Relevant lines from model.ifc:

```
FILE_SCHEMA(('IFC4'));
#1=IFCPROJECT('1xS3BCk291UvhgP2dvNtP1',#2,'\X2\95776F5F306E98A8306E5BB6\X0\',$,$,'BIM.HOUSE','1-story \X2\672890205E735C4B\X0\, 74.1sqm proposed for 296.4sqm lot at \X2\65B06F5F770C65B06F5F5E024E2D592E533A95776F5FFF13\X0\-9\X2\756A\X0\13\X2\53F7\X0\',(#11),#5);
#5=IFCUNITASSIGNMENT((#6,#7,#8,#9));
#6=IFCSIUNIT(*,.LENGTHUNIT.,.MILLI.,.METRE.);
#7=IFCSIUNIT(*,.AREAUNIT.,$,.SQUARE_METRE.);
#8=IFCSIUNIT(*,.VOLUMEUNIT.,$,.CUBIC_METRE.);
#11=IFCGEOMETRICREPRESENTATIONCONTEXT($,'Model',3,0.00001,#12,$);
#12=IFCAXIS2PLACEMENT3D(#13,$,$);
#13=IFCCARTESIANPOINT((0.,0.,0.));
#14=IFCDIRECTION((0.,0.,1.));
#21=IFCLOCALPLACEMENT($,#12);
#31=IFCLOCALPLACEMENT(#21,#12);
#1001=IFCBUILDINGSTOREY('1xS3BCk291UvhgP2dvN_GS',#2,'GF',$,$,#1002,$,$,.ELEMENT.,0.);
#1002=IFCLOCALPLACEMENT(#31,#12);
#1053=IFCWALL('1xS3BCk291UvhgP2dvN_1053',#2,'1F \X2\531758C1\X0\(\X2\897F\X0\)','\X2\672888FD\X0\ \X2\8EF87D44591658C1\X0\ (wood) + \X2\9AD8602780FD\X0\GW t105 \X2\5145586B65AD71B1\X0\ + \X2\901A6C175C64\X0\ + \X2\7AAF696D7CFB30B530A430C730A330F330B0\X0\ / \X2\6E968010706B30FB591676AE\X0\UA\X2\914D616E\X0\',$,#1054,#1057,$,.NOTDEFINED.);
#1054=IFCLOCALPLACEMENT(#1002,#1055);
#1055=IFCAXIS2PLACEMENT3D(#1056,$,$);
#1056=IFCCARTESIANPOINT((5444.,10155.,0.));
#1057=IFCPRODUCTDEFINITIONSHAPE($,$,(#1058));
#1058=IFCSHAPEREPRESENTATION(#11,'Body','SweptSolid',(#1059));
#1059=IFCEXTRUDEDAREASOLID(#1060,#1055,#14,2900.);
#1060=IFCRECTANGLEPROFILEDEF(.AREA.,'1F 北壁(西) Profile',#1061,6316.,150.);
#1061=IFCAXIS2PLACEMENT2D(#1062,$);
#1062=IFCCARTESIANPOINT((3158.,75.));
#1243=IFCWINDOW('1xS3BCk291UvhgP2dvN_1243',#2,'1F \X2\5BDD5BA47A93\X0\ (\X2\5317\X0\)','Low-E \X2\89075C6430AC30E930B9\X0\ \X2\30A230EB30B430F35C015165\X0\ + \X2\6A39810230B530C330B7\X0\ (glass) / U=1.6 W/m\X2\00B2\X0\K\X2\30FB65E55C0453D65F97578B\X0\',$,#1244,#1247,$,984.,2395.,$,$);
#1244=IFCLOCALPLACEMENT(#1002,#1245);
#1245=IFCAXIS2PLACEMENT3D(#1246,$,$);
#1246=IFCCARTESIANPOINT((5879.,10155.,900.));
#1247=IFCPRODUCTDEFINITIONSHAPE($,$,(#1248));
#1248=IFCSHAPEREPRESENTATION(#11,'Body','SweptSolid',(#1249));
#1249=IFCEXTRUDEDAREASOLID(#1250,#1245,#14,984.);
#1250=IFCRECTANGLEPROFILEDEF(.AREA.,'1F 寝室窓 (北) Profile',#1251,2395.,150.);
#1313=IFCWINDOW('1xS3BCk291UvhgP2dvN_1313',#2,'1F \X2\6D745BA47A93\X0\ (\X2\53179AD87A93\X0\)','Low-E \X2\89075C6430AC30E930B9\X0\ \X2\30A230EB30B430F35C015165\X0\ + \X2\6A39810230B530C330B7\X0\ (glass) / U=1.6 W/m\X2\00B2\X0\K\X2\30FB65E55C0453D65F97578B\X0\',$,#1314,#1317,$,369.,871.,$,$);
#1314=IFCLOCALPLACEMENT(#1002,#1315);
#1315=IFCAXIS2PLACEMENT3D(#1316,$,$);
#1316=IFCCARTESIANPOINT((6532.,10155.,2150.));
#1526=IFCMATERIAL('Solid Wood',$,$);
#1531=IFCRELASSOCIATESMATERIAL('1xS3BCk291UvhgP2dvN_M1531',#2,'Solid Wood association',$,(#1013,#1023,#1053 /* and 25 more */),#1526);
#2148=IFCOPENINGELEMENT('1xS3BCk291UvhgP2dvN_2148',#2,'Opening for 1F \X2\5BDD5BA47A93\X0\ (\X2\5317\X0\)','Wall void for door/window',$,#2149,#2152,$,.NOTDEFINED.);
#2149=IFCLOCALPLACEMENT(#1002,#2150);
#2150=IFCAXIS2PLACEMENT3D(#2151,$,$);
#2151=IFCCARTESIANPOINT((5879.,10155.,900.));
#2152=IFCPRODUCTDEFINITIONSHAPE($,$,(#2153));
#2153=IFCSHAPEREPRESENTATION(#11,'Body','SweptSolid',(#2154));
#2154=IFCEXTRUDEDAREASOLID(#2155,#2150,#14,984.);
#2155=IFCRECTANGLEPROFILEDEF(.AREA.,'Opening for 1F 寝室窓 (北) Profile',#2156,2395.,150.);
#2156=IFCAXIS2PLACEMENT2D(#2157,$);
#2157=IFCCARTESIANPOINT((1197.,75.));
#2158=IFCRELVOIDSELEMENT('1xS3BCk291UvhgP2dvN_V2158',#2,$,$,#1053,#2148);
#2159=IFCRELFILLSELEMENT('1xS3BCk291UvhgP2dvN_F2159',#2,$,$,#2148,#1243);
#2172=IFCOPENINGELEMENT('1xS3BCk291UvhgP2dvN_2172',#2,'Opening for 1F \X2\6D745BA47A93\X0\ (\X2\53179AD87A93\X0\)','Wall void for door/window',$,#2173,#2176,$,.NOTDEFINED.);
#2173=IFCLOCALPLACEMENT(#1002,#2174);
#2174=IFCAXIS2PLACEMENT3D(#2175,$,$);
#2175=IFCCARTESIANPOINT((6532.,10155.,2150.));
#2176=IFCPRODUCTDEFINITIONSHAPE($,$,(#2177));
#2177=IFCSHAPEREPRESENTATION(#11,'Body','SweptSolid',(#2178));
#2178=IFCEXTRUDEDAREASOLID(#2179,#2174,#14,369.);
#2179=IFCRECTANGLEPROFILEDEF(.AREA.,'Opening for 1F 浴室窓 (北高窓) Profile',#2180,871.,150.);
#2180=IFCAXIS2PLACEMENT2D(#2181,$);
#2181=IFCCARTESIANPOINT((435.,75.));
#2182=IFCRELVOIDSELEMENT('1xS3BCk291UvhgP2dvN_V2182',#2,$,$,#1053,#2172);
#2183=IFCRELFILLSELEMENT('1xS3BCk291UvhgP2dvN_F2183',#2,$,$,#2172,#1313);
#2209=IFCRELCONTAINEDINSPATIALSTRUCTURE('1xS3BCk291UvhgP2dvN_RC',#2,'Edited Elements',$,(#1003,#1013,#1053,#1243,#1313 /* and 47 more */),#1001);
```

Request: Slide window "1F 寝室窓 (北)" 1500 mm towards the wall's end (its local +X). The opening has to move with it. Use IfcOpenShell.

```python
import ifcopenshell
import ifcopenshell.api.geometry
import ifcopenshell.util.placement

model = ifcopenshell.open("model.ifc")

window = model.by_guid("1xS3BCk291UvhgP2dvN_1243")
opening = window.FillsVoids[0].RelatingOpeningElement
wall = opening.VoidsElements[0].RelatingBuildingElement

wall_matrix = ifcopenshell.util.placement.get_local_placement(wall.ObjectPlacement)
shift = wall_matrix[:3, 0] * 1500.0
before = ifcopenshell.util.placement.get_local_placement(window.ObjectPlacement)[:3, 3].copy()

# The window is not placed relative to its opening, so move both.
for product in (opening, window):
    matrix = ifcopenshell.util.placement.get_local_placement(product.ObjectPlacement)
    matrix[:3, 3] += shift
    ifcopenshell.api.geometry.edit_object_placement(model, product=product, matrix=matrix, is_si=False)

after = ifcopenshell.util.placement.get_local_placement(window.ObjectPlacement)[:3, 3]
print("window moved by", (after - before).round(3) + 0.0)

model.write("model_v2.ifc")
```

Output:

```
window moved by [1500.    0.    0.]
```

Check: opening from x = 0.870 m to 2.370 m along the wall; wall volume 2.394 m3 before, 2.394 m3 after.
